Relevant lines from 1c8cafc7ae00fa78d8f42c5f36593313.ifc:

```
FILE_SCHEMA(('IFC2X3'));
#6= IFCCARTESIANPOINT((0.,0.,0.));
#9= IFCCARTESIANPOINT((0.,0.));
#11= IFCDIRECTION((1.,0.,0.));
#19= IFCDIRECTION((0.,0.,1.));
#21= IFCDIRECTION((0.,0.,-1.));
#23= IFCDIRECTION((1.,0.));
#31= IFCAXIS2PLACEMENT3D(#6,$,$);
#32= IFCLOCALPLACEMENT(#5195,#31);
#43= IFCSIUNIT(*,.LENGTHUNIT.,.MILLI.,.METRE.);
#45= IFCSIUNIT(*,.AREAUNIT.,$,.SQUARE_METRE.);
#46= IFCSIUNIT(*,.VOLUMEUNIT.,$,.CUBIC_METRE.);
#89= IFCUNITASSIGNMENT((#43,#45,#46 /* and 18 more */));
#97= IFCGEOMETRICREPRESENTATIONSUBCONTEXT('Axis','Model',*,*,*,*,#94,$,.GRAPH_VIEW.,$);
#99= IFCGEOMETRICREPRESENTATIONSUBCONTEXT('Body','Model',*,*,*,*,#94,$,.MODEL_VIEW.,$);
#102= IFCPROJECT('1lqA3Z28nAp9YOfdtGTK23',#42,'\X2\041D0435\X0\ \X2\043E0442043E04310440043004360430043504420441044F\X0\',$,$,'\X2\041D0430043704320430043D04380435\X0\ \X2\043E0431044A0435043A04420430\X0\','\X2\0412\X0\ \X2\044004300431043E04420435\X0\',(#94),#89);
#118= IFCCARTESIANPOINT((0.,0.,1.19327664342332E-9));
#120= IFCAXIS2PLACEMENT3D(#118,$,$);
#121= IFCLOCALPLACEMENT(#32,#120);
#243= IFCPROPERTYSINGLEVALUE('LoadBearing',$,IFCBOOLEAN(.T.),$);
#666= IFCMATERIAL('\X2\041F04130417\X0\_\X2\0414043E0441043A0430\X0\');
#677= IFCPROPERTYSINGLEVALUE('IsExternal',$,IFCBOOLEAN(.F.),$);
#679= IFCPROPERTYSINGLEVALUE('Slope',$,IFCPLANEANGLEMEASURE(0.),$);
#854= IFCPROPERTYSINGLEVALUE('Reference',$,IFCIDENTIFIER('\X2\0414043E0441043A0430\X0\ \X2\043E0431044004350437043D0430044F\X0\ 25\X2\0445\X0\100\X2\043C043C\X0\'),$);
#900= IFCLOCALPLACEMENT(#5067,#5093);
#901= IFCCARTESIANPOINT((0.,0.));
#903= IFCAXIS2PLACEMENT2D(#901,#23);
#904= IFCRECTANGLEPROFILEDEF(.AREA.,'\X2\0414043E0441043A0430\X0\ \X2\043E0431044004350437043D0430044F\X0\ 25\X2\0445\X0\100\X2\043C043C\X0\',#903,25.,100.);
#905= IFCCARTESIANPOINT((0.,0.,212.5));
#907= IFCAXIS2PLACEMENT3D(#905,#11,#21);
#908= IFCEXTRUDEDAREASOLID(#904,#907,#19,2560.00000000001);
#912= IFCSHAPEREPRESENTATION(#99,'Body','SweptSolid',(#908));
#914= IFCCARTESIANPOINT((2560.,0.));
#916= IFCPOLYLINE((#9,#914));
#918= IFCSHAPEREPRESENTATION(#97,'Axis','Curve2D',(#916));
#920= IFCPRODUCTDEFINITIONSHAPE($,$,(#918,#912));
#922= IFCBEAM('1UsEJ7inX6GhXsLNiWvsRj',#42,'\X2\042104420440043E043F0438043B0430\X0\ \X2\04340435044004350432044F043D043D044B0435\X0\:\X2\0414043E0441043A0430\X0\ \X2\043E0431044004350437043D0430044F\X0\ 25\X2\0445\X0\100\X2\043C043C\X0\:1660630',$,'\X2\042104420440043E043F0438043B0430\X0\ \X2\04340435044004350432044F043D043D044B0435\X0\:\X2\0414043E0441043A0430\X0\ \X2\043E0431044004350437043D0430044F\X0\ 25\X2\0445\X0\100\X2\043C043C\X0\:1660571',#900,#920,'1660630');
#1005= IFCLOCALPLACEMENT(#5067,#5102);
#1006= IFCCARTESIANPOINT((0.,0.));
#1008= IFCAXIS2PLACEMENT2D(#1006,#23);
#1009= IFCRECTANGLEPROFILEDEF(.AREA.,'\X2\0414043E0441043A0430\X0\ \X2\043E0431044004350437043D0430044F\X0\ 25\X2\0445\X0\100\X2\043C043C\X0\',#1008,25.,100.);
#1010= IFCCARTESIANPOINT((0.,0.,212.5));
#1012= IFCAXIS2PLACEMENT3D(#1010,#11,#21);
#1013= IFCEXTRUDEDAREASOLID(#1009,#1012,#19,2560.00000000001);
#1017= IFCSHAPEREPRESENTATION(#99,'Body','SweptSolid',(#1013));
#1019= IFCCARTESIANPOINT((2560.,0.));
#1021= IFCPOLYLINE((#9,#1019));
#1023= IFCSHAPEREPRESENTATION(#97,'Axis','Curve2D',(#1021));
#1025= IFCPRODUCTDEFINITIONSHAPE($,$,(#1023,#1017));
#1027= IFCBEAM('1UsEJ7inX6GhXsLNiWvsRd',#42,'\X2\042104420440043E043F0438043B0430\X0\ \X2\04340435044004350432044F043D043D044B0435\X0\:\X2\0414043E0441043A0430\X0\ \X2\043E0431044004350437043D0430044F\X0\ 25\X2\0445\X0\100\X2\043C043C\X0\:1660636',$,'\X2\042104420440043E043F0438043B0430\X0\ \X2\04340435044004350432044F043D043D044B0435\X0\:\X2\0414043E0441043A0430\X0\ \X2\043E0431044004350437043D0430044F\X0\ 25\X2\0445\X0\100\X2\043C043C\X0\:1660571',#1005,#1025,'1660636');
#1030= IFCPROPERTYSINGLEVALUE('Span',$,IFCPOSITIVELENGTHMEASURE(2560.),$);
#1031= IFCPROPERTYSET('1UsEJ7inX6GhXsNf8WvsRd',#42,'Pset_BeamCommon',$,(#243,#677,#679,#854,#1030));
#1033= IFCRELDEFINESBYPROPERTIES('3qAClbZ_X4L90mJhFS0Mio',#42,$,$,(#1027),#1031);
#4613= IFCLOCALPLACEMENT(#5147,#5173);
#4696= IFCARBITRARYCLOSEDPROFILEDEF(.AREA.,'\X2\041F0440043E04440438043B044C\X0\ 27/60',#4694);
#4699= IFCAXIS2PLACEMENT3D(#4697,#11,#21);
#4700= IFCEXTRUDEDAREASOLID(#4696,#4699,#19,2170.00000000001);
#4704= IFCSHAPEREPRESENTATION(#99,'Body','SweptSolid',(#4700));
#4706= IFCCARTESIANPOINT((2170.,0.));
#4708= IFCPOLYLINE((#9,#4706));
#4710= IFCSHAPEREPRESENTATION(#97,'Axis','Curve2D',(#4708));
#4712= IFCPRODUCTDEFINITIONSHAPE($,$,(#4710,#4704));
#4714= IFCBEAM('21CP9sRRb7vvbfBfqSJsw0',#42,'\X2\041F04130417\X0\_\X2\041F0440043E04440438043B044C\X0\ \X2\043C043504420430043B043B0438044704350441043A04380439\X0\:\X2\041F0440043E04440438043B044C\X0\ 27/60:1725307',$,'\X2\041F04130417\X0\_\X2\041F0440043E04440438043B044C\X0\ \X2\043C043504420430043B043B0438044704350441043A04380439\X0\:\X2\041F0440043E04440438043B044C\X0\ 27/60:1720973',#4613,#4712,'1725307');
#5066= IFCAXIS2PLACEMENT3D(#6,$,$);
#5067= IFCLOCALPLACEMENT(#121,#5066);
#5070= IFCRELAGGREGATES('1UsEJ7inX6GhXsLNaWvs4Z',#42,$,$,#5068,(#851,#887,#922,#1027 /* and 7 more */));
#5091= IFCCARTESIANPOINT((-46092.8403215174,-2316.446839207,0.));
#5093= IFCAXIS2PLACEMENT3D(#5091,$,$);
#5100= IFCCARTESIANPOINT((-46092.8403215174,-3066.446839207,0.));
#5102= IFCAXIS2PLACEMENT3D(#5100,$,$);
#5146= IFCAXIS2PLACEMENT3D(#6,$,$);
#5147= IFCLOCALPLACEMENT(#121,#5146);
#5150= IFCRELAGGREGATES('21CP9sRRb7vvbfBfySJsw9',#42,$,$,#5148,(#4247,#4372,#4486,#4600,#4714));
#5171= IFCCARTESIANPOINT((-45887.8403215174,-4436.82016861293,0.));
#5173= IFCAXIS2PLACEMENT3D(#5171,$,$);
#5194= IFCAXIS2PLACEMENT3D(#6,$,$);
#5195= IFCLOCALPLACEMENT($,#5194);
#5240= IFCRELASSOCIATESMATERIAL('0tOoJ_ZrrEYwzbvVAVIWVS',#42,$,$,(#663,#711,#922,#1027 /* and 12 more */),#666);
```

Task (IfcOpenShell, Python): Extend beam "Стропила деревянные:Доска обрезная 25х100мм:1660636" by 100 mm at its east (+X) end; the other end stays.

```python
import numpy as np
import ifcopenshell
import ifcopenshell.api.pset
import ifcopenshell.util.element
import ifcopenshell.util.representation
import ifcopenshell.util.unit

model = ifcopenshell.open("1c8cafc7ae00fa78d8f42c5f36593313.ifc")
unit_scale = ifcopenshell.util.unit.calculate_unit_scale(model)

member = model.by_guid("1UsEJ7inX6GhXsLNiWvsRd")
change = 0.1 / unit_scale

# The extrusion runs towards the end named, so only its depth changes.
body = ifcopenshell.util.representation.get_representation(member, "Model", "Body")
solid = body.Items[0]
old_length = solid.Depth
solid.Depth += change

# Move the axis end point with it.
axis = next(r for r in member.Representation.Representations if r.RepresentationIdentifier == "Axis").Items[0]
start, end = (np.array(p.Coordinates) for p in axis.Points)
end = end + (end - start) / np.linalg.norm(end - start) * change
point = model.createIfcCartesianPoint(end.tolist())
axis.Points = [axis.Points[0], point]

# Update the stored length and volume.
pset = model.by_id(ifcopenshell.util.element.get_pset(member, "Pset_BeamCommon", should_inherit=False)["id"])
ifcopenshell.api.pset.edit_pset(model, pset=pset, properties={
    "Span": model.create_entity("IfcPositiveLengthMeasure", solid.Depth),
})

print(f"length {old_length:g} -> {solid.Depth:g}")

model.write("1c8cafc7ae00fa78d8f42c5f36593313_updated.ifc")
```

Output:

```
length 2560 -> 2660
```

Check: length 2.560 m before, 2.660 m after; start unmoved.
